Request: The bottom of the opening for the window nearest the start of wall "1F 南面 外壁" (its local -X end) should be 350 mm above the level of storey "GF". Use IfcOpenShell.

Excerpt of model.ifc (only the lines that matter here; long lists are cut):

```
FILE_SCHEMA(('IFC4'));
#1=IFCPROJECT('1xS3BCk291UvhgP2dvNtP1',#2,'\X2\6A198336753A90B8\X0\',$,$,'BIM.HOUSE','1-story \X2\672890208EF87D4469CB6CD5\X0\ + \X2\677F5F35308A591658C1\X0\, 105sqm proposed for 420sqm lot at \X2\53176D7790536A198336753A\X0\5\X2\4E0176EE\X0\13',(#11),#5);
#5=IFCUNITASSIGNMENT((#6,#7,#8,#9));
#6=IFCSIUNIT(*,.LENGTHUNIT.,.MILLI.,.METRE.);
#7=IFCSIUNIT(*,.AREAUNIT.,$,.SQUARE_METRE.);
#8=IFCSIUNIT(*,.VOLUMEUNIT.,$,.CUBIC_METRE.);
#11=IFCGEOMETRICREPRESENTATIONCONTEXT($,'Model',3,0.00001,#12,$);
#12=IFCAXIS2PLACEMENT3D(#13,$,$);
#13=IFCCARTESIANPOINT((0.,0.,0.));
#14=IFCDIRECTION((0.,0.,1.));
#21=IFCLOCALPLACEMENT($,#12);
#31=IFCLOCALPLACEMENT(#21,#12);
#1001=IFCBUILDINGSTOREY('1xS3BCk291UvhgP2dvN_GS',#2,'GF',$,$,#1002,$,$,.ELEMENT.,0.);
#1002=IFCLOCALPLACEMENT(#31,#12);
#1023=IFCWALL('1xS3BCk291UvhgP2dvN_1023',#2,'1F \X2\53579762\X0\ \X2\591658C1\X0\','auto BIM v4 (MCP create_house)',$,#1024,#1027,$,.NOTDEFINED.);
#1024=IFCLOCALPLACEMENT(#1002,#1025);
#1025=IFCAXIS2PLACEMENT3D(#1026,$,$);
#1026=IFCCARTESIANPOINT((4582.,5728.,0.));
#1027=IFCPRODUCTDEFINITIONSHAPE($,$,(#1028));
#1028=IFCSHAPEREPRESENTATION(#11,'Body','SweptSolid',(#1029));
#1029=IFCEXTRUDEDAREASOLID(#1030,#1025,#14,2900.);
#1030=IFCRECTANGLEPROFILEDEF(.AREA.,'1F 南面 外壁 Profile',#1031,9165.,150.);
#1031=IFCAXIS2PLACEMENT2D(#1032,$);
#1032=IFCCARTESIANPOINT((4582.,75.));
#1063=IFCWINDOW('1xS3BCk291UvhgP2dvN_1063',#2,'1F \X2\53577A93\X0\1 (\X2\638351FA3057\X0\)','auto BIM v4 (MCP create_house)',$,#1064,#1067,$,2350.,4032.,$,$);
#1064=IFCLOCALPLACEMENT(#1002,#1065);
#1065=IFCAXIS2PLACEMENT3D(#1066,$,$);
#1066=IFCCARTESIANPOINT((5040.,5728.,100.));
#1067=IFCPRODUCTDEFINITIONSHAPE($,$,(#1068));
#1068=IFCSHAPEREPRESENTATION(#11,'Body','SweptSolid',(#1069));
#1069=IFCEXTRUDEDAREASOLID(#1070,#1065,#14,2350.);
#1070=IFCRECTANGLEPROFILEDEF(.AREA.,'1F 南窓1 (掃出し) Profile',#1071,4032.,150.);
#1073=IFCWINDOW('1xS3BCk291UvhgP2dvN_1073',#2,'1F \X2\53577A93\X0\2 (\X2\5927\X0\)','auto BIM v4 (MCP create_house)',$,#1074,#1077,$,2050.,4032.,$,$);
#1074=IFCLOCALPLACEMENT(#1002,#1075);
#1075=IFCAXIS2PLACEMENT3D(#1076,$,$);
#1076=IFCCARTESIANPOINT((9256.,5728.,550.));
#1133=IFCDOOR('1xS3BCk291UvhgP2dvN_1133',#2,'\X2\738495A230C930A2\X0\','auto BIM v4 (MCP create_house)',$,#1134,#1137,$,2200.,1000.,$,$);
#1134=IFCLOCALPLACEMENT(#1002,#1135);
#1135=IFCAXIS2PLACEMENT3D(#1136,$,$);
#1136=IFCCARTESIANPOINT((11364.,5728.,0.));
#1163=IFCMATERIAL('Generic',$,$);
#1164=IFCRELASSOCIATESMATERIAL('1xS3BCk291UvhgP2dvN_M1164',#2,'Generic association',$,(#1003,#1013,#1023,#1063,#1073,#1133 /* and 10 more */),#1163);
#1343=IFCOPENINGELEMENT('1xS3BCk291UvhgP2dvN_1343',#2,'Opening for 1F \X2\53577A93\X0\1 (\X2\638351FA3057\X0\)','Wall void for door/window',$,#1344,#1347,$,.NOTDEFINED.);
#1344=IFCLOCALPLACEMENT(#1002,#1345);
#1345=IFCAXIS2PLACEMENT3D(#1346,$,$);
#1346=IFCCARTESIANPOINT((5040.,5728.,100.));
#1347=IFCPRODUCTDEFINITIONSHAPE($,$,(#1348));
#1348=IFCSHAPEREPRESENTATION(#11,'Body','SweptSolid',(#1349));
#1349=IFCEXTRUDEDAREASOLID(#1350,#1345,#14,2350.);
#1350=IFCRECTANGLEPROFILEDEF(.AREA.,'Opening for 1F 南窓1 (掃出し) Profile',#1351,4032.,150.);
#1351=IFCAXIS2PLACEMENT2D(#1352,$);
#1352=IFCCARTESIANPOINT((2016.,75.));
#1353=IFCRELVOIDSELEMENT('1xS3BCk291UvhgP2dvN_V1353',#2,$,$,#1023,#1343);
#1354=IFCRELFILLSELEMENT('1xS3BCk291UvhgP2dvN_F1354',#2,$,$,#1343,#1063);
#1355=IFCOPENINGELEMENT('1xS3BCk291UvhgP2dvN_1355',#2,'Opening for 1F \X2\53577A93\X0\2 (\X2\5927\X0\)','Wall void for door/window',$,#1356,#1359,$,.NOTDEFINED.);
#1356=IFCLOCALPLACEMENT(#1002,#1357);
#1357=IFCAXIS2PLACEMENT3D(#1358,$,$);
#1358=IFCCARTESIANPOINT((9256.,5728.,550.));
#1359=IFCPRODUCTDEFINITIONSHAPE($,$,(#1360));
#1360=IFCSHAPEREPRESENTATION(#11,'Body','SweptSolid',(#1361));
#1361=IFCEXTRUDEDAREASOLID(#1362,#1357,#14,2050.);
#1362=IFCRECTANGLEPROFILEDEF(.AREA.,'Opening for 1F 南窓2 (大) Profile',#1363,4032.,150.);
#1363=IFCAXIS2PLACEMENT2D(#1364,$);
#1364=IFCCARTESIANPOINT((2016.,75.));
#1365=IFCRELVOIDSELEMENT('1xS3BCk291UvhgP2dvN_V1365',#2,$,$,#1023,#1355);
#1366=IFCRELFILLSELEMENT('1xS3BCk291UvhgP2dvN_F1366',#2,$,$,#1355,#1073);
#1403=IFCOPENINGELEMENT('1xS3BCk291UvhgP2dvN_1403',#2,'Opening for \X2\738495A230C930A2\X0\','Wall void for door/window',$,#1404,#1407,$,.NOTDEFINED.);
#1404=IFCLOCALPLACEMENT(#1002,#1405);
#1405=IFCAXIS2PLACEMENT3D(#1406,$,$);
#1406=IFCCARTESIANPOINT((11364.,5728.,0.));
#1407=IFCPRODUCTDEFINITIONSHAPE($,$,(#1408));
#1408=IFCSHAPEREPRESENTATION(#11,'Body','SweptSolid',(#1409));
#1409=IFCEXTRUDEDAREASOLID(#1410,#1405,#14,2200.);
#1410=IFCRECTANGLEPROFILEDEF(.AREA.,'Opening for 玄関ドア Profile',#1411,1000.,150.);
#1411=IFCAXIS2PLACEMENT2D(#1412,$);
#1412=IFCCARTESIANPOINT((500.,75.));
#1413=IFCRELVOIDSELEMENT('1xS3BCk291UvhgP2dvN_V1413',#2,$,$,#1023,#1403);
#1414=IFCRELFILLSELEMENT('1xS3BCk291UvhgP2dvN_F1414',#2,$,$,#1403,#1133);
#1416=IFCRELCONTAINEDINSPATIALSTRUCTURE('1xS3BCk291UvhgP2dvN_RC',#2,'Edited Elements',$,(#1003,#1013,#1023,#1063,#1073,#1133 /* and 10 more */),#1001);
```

```python
import numpy as np
import ifcopenshell
import ifcopenshell.api.geometry
import ifcopenshell.geom
import ifcopenshell.util.element
import ifcopenshell.util.placement
import ifcopenshell.util.shape
import ifcopenshell.util.unit

model = ifcopenshell.open("model.ifc")
unit_scale = ifcopenshell.util.unit.calculate_unit_scale(model)

window = model.by_guid("1xS3BCk291UvhgP2dvN_1063")
opening = window.FillsVoids[0].RelatingOpeningElement
storey = ifcopenshell.util.element.get_container(window, ifc_class="IfcBuildingStorey")
level = ifcopenshell.util.placement.get_local_placement(storey.ObjectPlacement)[2, 3]

# The opening's origin need not be at the sill, so measure its lowest point.
shape = ifcopenshell.geom.create_shape(ifcopenshell.geom.settings(), opening)
bottom = ifcopenshell.util.shape.get_shape_bottom_elevation(shape, shape.geometry) / unit_scale
dz = level + 350.0 - bottom

shift = np.array([0.0, 0.0, dz])
# The window is not placed relative to its opening, so move both.
for product in (opening, window):
    matrix = ifcopenshell.util.placement.get_local_placement(product.ObjectPlacement)
    matrix[:3, 3] += shift
    ifcopenshell.api.geometry.edit_object_placement(model, product=product, matrix=matrix, is_si=False)

print(f"moved by {dz * unit_scale:+.3f} m")

model.write("model_v2.ifc")
```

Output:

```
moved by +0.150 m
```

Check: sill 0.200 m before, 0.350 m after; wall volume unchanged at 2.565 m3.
